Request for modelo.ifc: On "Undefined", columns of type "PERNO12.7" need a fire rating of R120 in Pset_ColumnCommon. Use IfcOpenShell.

First a look at what the model holds.

```python
import ifcopenshell
import ifcopenshell.util.element

model = ifcopenshell.open("modelo.ifc")
print(model.schema)
storey = next(s for s in model.by_type("IfcBuildingStorey") if s.Name == "Undefined")
columns = [e for e in ifcopenshell.util.element.get_decomposition(storey) if e.is_a("IfcColumn")]
seen = {}
for e in columns:
    element_type = ifcopenshell.util.element.get_type(e)
    key = (element_type.Name if element_type != e and element_type else None, ifcopenshell.util.element.get_pset(e, "Pset_ColumnCommon", "FireRating"))
    seen[key] = seen.get(key, 0) + 1
for (name, value), count in sorted(seen.items(), key=str):
    print(count, "x", name, "|", value)
```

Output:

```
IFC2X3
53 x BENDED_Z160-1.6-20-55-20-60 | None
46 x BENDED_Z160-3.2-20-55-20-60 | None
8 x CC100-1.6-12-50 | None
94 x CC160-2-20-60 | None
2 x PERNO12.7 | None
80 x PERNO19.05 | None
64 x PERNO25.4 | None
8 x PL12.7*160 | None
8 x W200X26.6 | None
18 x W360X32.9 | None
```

```python
import ifcopenshell
import ifcopenshell.api.pset
import ifcopenshell.util.element

model = ifcopenshell.open("modelo.ifc")

storey = next(s for s in model.by_type("IfcBuildingStorey") if s.Name == "Undefined")
columns = [e for e in ifcopenshell.util.element.get_decomposition(storey) if e.is_a("IfcColumn")]

count = 0
for e in columns:
    element_type = ifcopenshell.util.element.get_type(e)
    if element_type in (None, e) or element_type.Name != "PERNO12.7":
        continue
    found = ifcopenshell.util.element.get_pset(e, "Pset_ColumnCommon", should_inherit=False)
    if found:
        pset = model.by_id(found["id"])
        if len(ifcopenshell.util.element.get_elements_by_pset(pset)) > 1:
            pset = ifcopenshell.api.pset.unshare_pset(model, products=[e], pset=pset)[0]
    else:
        pset = ifcopenshell.api.pset.add_pset(model, product=e, name="Pset_ColumnCommon")
    ifcopenshell.api.pset.edit_pset(model, pset=pset, properties={"FireRating": "R120"})
    count += 1

print(count, "columns updated")

model.write("modelo_rev.ifc")
```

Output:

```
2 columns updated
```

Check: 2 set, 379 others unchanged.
